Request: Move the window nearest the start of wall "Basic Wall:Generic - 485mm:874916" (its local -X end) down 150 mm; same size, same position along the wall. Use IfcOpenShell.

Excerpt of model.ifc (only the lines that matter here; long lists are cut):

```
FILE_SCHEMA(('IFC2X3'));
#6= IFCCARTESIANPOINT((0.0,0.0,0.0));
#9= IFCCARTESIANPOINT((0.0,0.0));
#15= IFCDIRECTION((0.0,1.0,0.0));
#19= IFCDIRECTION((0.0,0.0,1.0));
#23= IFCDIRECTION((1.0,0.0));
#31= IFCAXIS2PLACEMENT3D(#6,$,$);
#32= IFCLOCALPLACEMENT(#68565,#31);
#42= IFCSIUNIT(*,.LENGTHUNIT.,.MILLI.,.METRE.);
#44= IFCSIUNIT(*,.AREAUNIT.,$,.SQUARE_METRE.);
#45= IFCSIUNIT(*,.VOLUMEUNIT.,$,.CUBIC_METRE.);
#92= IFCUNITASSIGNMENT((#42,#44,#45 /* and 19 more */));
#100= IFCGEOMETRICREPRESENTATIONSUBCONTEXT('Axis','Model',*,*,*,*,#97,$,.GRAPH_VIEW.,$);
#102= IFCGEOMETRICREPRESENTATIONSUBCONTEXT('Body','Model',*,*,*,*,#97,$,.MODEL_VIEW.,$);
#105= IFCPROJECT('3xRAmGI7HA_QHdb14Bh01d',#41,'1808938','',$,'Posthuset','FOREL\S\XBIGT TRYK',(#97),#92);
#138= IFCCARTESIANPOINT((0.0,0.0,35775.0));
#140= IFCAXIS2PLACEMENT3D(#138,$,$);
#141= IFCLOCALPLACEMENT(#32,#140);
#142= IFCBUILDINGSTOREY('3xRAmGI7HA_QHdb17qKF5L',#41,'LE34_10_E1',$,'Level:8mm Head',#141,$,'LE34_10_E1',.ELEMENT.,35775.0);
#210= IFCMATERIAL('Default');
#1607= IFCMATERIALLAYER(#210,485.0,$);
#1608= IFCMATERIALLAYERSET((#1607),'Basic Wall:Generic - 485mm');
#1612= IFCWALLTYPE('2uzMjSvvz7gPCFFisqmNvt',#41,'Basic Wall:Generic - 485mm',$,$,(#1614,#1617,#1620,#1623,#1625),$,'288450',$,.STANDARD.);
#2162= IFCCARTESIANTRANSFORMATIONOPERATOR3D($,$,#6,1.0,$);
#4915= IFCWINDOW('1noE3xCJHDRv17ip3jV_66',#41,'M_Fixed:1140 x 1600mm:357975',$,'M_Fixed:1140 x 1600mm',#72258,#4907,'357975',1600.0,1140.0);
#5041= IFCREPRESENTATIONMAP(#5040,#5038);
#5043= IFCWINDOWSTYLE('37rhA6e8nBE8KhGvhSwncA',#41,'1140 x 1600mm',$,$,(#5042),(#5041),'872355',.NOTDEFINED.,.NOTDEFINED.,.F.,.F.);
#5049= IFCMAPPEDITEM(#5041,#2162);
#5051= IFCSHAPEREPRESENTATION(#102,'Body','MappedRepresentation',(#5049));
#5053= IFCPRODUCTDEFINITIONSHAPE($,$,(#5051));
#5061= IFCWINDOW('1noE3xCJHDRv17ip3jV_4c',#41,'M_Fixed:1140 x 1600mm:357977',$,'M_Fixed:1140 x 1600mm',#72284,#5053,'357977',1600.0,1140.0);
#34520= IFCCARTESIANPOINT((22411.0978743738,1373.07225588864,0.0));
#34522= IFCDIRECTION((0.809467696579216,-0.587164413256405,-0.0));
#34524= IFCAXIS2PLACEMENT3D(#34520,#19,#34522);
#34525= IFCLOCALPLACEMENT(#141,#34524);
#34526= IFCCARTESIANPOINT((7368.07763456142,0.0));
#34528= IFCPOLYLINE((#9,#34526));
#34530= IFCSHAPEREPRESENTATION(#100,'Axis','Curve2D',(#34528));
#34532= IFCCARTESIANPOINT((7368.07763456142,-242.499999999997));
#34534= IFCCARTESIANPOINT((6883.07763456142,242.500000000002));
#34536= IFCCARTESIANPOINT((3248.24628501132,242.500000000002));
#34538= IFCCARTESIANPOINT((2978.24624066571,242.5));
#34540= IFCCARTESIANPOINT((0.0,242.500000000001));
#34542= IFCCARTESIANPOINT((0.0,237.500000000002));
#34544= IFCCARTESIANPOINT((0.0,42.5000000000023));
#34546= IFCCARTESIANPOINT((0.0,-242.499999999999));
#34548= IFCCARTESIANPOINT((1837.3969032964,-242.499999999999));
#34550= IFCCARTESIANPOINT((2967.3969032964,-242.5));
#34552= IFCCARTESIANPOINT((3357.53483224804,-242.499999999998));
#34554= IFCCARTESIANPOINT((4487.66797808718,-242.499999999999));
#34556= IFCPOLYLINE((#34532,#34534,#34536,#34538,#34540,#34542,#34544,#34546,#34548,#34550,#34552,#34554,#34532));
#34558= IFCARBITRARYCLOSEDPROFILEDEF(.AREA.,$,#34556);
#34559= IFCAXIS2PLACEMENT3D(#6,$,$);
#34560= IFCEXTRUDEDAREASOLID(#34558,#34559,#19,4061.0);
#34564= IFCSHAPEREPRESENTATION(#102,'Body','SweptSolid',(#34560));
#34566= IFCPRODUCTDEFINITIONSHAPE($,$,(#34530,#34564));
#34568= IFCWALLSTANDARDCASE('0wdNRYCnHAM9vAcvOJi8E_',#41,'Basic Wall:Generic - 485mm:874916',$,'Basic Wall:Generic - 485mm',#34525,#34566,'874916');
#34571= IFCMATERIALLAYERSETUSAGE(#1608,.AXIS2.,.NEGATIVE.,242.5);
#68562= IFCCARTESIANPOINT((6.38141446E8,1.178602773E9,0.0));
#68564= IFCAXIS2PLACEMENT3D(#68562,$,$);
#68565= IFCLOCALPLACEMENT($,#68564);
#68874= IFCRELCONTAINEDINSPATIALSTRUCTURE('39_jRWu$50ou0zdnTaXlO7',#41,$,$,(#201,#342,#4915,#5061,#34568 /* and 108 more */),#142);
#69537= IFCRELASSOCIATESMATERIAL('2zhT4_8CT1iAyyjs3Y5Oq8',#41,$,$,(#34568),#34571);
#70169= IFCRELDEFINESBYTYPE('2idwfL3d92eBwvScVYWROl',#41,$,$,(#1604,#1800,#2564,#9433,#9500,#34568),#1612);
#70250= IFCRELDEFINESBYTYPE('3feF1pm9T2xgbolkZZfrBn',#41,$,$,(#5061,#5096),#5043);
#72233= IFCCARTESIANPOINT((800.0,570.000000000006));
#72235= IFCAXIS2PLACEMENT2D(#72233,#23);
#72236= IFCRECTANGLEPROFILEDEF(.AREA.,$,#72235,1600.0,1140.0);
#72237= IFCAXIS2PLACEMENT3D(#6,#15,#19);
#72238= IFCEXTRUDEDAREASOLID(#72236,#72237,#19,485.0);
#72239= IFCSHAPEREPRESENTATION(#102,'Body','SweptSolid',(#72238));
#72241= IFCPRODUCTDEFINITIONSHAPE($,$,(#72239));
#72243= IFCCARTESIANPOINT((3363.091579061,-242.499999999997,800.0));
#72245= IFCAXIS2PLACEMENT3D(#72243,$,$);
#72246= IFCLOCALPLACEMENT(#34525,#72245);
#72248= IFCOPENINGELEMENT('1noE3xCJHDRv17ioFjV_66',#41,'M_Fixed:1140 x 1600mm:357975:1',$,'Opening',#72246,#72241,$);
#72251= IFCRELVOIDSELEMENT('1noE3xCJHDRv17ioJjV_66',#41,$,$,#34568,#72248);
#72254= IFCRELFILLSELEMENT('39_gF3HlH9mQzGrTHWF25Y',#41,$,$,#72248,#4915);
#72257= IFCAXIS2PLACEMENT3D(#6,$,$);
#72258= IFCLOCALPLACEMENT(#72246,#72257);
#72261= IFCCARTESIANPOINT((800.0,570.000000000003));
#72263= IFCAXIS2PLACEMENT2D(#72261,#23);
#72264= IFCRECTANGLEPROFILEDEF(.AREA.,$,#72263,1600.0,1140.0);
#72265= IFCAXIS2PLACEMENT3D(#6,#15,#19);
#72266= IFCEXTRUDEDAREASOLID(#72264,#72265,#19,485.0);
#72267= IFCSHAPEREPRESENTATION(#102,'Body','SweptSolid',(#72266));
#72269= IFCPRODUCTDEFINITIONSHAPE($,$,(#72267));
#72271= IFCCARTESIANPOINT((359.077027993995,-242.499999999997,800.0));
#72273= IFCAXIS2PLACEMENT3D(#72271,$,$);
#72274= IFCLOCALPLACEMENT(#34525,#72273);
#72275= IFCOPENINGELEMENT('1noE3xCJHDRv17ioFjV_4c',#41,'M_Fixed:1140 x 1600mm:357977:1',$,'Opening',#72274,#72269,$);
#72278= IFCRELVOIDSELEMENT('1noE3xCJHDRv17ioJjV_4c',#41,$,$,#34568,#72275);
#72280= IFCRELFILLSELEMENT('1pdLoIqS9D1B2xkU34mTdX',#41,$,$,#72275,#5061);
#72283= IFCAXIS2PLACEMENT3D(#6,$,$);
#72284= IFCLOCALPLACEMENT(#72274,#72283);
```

```python
import numpy as np
import ifcopenshell
import ifcopenshell.api.geometry
import ifcopenshell.util.placement
import ifcopenshell.util.unit

model = ifcopenshell.open("model.ifc")
unit_scale = ifcopenshell.util.unit.calculate_unit_scale(model)

window = model.by_guid("1noE3xCJHDRv17ip3jV_4c")
opening = window.FillsVoids[0].RelatingOpeningElement
dz = -0.15 / unit_scale

shift = np.array([0.0, 0.0, dz])
# The window is placed relative to its opening, so it follows when the opening moves.
matrix = ifcopenshell.util.placement.get_local_placement(opening.ObjectPlacement)
matrix[:3, 3] += shift
ifcopenshell.api.geometry.edit_object_placement(
    model, product=opening, matrix=matrix, is_si=False, should_transform_children=True
)

print(f"moved by {dz * unit_scale:+.3f} m")

model.write("model_v2.ifc")
```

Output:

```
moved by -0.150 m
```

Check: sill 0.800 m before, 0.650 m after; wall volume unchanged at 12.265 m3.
